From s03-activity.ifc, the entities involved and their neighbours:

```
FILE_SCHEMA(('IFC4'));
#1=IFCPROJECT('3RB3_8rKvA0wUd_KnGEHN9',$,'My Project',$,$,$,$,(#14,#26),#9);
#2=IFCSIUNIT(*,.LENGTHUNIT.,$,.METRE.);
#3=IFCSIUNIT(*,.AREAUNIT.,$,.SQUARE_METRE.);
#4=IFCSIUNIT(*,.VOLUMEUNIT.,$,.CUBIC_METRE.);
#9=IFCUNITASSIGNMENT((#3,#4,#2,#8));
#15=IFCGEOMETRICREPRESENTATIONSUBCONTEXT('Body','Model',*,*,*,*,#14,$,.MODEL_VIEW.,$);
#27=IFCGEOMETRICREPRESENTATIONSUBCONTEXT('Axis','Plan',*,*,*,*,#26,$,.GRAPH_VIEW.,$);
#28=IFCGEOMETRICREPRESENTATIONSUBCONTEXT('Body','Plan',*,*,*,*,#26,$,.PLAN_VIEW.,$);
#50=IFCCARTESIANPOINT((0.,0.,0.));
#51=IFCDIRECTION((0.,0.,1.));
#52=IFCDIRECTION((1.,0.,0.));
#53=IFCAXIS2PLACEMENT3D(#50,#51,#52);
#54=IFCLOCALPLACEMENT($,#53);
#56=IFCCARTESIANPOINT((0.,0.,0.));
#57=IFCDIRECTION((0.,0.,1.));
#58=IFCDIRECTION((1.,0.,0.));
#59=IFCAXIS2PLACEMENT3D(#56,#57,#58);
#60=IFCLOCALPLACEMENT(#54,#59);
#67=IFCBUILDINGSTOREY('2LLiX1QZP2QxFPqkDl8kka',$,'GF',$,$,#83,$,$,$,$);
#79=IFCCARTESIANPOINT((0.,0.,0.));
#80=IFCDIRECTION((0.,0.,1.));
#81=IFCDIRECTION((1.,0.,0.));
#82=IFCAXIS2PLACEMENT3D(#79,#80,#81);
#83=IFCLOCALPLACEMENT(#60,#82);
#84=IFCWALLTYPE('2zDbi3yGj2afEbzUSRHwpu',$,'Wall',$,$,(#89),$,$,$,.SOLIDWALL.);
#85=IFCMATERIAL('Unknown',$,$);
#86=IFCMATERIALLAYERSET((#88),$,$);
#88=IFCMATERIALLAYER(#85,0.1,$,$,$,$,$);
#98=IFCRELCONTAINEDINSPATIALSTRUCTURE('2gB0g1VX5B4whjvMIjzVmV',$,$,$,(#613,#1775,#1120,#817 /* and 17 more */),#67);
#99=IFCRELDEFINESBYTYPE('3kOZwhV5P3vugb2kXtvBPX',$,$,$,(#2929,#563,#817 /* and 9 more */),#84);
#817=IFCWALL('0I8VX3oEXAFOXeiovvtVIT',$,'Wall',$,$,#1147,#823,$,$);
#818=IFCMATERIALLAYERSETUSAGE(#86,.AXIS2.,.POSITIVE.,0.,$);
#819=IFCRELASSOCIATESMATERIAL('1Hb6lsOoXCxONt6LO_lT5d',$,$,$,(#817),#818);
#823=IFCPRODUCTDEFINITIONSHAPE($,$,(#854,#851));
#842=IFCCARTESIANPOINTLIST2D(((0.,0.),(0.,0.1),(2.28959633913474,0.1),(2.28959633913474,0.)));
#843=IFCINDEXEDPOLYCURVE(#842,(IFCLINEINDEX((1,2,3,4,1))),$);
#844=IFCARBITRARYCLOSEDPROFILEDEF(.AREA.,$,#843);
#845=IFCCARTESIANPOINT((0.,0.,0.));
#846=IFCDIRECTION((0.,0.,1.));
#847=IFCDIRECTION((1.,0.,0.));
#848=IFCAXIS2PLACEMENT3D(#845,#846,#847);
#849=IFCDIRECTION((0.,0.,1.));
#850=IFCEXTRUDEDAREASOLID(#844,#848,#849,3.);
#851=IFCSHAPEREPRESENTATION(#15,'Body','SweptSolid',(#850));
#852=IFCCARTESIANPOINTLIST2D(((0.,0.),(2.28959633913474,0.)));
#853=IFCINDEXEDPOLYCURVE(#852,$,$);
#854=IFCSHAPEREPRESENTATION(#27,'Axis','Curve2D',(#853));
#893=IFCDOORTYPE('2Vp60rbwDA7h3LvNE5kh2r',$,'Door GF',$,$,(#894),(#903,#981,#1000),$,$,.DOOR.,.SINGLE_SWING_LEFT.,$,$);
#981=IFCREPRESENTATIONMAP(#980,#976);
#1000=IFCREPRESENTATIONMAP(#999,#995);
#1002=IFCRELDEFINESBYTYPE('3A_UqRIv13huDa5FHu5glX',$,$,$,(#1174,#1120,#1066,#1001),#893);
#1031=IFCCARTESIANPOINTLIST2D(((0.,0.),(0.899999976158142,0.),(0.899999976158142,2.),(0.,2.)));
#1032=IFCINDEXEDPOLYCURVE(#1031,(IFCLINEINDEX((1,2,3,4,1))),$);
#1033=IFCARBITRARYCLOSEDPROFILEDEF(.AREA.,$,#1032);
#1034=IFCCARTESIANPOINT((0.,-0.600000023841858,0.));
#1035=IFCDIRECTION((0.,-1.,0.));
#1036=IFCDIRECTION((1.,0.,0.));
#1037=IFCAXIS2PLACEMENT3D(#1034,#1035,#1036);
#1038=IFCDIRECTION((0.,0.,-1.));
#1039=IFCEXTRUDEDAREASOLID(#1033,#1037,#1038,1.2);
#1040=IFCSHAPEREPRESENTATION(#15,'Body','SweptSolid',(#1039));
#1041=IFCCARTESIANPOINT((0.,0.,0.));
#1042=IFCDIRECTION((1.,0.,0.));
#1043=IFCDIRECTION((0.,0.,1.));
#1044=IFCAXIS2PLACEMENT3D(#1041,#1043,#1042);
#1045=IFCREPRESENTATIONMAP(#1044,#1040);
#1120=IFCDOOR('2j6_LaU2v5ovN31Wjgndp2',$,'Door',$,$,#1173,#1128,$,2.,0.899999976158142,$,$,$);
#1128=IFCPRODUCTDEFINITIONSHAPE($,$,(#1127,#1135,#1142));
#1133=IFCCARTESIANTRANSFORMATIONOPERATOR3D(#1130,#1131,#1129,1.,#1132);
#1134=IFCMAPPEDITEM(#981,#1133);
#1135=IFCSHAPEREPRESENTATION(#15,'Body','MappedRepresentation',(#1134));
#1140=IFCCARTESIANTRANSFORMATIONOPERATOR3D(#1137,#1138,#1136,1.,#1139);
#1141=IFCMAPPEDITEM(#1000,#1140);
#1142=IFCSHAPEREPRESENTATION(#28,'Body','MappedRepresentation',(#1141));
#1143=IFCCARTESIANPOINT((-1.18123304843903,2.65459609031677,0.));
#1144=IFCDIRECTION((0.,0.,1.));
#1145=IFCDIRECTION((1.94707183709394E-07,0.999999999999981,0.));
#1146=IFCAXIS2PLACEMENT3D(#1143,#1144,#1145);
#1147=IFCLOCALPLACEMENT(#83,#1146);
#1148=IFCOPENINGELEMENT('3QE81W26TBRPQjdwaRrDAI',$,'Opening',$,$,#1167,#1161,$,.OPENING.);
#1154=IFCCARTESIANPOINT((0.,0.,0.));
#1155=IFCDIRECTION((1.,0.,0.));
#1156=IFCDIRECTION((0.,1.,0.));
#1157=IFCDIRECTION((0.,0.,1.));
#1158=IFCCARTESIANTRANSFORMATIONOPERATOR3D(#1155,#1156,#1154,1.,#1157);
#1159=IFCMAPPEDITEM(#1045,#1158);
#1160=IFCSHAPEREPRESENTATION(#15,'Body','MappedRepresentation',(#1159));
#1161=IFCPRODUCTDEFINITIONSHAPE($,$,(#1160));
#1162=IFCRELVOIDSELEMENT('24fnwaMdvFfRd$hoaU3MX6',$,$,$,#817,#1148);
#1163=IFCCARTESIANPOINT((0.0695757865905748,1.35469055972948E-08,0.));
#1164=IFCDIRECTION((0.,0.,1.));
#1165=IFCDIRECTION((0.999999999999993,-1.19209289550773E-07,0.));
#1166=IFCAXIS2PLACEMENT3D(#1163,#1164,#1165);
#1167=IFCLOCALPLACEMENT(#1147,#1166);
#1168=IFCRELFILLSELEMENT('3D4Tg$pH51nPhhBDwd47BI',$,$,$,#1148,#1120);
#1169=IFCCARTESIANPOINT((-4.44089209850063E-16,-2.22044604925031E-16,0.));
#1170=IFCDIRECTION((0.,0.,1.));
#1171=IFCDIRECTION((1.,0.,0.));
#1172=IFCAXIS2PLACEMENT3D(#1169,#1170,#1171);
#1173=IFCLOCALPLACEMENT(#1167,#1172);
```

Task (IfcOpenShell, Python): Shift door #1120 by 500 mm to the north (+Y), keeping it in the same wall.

```python
import ifcopenshell
import ifcopenshell.api.geometry
import ifcopenshell.util.placement

model = ifcopenshell.open("s03-activity.ifc")

door = model.by_guid("2j6_LaU2v5ovN31Wjgndp2")
opening = door.FillsVoids[0].RelatingOpeningElement
wall = opening.VoidsElements[0].RelatingBuildingElement

wall_matrix = ifcopenshell.util.placement.get_local_placement(wall.ObjectPlacement)
shift = wall_matrix[:3, 0] * 0.5
before = ifcopenshell.util.placement.get_local_placement(door.ObjectPlacement)[:3, 3].copy()

# The door is placed relative to its opening, so it follows when the opening moves.
matrix = ifcopenshell.util.placement.get_local_placement(opening.ObjectPlacement)
matrix[:3, 3] += shift
ifcopenshell.api.geometry.edit_object_placement(
    model, product=opening, matrix=matrix, is_si=False, should_transform_children=True
)

after = ifcopenshell.util.placement.get_local_placement(door.ObjectPlacement)[:3, 3]
print("door moved by", (after - before).round(3) + 0.0)

model.write("s03-activity-out.ifc")
```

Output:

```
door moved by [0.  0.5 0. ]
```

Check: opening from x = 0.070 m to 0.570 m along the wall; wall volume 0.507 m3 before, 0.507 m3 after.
